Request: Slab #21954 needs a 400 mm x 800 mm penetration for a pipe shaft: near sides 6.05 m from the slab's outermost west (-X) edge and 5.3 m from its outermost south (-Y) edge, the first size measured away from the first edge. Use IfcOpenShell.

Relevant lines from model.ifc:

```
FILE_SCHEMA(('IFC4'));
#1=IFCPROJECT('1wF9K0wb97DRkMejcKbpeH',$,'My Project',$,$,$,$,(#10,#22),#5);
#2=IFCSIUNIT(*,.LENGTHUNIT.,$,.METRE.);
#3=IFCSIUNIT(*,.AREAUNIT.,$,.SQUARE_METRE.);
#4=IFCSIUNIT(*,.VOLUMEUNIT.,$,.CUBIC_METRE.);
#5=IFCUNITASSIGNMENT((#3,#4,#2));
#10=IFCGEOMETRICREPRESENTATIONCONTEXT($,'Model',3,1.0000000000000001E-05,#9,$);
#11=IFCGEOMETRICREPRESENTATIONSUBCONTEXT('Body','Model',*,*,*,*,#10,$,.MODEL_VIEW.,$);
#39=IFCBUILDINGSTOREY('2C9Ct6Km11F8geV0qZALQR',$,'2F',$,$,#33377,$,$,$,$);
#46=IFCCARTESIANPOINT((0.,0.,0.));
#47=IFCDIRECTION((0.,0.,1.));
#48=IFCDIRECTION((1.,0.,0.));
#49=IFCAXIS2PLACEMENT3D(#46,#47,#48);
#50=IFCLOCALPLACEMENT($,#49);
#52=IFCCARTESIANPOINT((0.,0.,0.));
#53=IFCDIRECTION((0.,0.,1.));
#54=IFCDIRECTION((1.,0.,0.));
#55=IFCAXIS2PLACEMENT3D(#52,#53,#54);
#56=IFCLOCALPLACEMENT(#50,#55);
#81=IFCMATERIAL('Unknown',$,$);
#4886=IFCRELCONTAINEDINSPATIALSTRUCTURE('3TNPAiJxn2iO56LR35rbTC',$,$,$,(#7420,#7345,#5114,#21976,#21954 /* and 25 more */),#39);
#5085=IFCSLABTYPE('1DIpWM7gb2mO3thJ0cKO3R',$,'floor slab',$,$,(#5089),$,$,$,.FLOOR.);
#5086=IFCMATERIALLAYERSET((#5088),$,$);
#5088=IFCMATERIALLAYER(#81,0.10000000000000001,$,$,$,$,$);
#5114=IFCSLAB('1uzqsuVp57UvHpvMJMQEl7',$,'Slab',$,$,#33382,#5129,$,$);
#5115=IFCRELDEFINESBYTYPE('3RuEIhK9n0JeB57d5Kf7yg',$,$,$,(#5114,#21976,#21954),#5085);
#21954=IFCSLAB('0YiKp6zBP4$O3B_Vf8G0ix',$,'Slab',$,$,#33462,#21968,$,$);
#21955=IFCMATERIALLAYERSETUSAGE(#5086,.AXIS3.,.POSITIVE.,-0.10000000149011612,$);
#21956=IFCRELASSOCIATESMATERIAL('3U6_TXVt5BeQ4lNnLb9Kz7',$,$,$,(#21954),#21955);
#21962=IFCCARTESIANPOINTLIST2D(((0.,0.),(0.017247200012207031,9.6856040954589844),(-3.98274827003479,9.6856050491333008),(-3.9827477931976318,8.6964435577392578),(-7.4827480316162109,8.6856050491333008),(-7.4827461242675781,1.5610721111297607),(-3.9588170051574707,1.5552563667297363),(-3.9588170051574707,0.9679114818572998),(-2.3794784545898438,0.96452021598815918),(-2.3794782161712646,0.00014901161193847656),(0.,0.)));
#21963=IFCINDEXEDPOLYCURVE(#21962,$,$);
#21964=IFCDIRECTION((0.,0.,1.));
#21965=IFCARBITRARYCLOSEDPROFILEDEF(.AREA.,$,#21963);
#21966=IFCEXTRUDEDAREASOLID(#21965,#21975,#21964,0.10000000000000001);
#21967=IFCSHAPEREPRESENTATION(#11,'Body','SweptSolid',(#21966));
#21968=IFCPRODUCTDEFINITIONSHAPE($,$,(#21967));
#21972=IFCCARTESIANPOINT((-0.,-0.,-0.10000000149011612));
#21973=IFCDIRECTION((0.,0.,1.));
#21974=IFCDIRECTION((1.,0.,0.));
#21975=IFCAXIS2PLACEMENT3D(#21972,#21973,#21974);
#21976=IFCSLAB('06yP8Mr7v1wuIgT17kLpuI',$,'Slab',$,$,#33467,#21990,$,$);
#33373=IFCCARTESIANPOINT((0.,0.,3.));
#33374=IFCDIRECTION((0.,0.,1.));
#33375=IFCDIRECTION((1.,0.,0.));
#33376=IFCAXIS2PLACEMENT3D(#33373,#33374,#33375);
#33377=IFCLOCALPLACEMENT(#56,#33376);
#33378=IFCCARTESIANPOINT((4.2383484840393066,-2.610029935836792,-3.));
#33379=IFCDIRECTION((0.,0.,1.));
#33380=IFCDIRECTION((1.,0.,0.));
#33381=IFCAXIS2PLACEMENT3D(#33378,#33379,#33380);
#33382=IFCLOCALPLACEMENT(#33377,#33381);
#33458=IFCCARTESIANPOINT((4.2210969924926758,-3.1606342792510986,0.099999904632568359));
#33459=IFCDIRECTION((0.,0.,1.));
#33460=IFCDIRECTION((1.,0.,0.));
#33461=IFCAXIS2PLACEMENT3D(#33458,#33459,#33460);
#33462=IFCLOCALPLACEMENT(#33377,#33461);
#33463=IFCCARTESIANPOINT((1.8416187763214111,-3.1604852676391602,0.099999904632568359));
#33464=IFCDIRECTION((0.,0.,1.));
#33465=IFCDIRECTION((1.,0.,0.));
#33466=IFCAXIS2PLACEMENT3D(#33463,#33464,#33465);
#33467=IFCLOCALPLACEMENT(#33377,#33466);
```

```python
import numpy as np
import ifcopenshell
import ifcopenshell.api.feature
import ifcopenshell.api.geometry
import ifcopenshell.api.root
import ifcopenshell.geom
import ifcopenshell.util.placement
import ifcopenshell.util.representation
import ifcopenshell.util.shape
import ifcopenshell.util.unit

model = ifcopenshell.open("model.ifc")
unit_scale = ifcopenshell.util.unit.calculate_unit_scale(model)
settings = ifcopenshell.geom.settings()


def volume(element):
    """Net volume in cubic metres, openings subtracted."""
    shape = ifcopenshell.geom.create_shape(settings, element)
    return ifcopenshell.util.shape.get_volume(shape.geometry)


slab = model.by_guid("0YiKp6zBP4$O3B_Vf8G0ix")
before = volume(slab)

# Extent in the slab's own axes, in metres. The edges named are its -X and -Y sides.
slab_shape = ifcopenshell.geom.create_shape(settings, slab)
vertices = ifcopenshell.util.shape.get_vertices(slab_shape.geometry)
x_min, y_min, bottom = vertices.min(axis=0)
top = vertices[:, 2].max()

opening = ifcopenshell.api.root.create_entity(model, ifc_class="IfcOpeningElement", name="Pipe shaft opening", predefined_type="OPENING")
context = ifcopenshell.util.representation.get_context(model, "Model", "Body", "MODEL_VIEW")
width, depth = 0.4, 0.8
outline = [(0.0, 0.0), (width, 0.0), (width, depth), (0.0, depth), (0.0, 0.0)]
# Overshoot both faces by 50 mm so the cut is clean.
shape = ifcopenshell.api.geometry.add_slab_representation(
    model, context=context, depth=top - bottom + 0.1, polyline=outline
)
ifcopenshell.api.geometry.assign_representation(model, product=opening, representation=shape)

matrix = ifcopenshell.util.placement.get_local_placement(slab.ObjectPlacement)
matrix[:, 3] = matrix @ np.append(np.array([x_min + 6.05, y_min + 5.3, bottom - 0.05]) / unit_scale, 1.0)
ifcopenshell.api.geometry.edit_object_placement(model, product=opening, matrix=matrix, is_si=False)
ifcopenshell.api.feature.add_feature(model, feature=opening, element=slab)

after = volume(slab)

print(f"slab volume {before:.3f} -> {after:.3f} m3")

model.write("model_edited.ifc")
```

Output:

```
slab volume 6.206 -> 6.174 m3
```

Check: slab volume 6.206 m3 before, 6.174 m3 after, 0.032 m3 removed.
